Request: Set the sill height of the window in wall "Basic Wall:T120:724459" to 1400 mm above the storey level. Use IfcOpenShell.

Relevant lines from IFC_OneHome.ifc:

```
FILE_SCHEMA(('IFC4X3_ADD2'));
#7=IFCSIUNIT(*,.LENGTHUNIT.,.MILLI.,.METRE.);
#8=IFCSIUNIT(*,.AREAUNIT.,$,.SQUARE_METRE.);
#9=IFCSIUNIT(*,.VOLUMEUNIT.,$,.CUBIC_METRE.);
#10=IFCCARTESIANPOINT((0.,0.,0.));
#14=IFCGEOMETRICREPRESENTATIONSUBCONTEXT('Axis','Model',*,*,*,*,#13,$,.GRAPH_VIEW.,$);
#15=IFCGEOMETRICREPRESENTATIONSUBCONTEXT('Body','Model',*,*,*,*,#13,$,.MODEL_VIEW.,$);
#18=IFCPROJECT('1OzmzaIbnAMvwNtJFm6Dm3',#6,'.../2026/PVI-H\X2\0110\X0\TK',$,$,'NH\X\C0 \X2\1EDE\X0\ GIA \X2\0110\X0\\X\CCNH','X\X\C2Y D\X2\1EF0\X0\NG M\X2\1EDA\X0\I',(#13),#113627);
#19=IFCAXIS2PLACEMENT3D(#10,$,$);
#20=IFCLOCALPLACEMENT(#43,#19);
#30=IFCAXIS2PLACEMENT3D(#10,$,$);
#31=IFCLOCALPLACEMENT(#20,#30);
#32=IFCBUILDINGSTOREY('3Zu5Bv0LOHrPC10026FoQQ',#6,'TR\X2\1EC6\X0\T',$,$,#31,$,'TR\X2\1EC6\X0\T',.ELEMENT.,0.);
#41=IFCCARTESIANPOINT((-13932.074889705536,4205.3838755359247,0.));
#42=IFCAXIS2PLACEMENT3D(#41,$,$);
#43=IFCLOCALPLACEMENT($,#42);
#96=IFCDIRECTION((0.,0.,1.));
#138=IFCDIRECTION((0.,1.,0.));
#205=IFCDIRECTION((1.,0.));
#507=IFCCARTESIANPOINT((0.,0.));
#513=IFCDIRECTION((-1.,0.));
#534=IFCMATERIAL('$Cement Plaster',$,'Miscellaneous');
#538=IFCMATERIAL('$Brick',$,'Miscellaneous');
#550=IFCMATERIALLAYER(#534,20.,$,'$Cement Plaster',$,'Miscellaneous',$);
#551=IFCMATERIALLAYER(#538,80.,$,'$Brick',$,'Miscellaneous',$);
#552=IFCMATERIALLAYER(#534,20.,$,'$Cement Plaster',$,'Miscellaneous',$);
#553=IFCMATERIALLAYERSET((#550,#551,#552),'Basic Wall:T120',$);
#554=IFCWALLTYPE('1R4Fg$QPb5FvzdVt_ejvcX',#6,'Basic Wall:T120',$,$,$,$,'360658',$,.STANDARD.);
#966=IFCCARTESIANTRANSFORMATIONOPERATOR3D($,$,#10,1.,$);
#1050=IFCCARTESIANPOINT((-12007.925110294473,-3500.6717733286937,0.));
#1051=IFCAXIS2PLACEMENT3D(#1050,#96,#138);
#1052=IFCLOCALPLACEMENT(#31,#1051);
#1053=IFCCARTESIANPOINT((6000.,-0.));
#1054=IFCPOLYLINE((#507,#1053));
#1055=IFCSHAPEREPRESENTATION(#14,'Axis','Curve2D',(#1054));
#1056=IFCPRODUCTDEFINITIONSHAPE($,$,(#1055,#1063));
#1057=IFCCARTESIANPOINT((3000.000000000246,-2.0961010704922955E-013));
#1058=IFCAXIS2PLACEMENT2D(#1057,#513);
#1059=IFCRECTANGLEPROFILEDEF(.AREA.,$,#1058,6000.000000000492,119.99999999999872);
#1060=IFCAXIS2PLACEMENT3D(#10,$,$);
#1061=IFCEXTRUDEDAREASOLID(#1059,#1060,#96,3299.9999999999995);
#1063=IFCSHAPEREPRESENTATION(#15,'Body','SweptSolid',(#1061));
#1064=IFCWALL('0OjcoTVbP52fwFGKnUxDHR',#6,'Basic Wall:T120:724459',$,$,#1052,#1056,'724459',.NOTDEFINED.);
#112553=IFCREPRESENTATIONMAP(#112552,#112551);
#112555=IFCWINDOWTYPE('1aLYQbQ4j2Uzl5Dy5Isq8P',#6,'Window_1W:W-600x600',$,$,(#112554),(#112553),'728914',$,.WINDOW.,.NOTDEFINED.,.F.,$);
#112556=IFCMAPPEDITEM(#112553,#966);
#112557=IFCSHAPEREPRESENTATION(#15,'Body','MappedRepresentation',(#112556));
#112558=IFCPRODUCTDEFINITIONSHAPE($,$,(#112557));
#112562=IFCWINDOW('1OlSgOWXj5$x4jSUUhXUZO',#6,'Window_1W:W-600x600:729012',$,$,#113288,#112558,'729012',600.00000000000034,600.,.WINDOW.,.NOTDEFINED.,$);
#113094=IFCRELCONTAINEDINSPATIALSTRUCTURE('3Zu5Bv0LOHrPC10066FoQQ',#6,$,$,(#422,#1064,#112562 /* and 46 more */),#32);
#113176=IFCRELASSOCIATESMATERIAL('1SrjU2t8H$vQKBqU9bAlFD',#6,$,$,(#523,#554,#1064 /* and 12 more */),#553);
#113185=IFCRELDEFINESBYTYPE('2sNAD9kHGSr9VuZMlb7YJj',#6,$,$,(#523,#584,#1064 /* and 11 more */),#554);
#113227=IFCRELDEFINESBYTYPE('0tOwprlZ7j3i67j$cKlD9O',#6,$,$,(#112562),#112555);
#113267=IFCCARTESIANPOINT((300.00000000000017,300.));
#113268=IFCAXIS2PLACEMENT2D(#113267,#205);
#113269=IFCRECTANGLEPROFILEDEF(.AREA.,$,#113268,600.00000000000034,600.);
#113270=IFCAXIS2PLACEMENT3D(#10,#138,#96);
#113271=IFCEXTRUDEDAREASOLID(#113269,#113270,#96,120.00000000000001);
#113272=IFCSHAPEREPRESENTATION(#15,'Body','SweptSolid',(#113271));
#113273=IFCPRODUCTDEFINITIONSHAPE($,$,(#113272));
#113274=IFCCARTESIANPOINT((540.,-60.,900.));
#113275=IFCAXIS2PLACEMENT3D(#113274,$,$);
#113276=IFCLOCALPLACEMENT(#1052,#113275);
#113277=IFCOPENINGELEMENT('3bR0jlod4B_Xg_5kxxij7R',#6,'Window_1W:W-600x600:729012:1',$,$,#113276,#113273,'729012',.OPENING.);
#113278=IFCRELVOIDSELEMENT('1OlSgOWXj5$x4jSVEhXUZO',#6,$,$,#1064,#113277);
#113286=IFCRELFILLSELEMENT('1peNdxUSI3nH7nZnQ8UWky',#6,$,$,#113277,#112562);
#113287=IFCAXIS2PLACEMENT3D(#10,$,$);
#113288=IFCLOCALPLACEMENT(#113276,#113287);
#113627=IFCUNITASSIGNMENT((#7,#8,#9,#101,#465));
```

```python
import numpy as np
import ifcopenshell
import ifcopenshell.api.geometry
import ifcopenshell.geom
import ifcopenshell.util.element
import ifcopenshell.util.placement
import ifcopenshell.util.shape
import ifcopenshell.util.unit

model = ifcopenshell.open("IFC_OneHome.ifc")
unit_scale = ifcopenshell.util.unit.calculate_unit_scale(model)

window = model.by_guid("1OlSgOWXj5$x4jSUUhXUZO")
opening = window.FillsVoids[0].RelatingOpeningElement
storey = ifcopenshell.util.element.get_container(window, ifc_class="IfcBuildingStorey")
level = ifcopenshell.util.placement.get_local_placement(storey.ObjectPlacement)[2, 3]

# The opening's origin need not be at the sill, so measure its lowest point.
shape = ifcopenshell.geom.create_shape(ifcopenshell.geom.settings(), opening)
bottom = ifcopenshell.util.shape.get_shape_bottom_elevation(shape, shape.geometry) / unit_scale
dz = level + 1.4 / unit_scale - bottom

shift = np.array([0.0, 0.0, dz])
# The window is placed relative to its opening, so it follows when the opening moves.
matrix = ifcopenshell.util.placement.get_local_placement(opening.ObjectPlacement)
matrix[:3, 3] += shift
ifcopenshell.api.geometry.edit_object_placement(
    model, product=opening, matrix=matrix, is_si=False, should_transform_children=True
)

print(f"moved by {dz * unit_scale:+.3f} m")

model.write("IFC_OneHome_updated.ifc")
```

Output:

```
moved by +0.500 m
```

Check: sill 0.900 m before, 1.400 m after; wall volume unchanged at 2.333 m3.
